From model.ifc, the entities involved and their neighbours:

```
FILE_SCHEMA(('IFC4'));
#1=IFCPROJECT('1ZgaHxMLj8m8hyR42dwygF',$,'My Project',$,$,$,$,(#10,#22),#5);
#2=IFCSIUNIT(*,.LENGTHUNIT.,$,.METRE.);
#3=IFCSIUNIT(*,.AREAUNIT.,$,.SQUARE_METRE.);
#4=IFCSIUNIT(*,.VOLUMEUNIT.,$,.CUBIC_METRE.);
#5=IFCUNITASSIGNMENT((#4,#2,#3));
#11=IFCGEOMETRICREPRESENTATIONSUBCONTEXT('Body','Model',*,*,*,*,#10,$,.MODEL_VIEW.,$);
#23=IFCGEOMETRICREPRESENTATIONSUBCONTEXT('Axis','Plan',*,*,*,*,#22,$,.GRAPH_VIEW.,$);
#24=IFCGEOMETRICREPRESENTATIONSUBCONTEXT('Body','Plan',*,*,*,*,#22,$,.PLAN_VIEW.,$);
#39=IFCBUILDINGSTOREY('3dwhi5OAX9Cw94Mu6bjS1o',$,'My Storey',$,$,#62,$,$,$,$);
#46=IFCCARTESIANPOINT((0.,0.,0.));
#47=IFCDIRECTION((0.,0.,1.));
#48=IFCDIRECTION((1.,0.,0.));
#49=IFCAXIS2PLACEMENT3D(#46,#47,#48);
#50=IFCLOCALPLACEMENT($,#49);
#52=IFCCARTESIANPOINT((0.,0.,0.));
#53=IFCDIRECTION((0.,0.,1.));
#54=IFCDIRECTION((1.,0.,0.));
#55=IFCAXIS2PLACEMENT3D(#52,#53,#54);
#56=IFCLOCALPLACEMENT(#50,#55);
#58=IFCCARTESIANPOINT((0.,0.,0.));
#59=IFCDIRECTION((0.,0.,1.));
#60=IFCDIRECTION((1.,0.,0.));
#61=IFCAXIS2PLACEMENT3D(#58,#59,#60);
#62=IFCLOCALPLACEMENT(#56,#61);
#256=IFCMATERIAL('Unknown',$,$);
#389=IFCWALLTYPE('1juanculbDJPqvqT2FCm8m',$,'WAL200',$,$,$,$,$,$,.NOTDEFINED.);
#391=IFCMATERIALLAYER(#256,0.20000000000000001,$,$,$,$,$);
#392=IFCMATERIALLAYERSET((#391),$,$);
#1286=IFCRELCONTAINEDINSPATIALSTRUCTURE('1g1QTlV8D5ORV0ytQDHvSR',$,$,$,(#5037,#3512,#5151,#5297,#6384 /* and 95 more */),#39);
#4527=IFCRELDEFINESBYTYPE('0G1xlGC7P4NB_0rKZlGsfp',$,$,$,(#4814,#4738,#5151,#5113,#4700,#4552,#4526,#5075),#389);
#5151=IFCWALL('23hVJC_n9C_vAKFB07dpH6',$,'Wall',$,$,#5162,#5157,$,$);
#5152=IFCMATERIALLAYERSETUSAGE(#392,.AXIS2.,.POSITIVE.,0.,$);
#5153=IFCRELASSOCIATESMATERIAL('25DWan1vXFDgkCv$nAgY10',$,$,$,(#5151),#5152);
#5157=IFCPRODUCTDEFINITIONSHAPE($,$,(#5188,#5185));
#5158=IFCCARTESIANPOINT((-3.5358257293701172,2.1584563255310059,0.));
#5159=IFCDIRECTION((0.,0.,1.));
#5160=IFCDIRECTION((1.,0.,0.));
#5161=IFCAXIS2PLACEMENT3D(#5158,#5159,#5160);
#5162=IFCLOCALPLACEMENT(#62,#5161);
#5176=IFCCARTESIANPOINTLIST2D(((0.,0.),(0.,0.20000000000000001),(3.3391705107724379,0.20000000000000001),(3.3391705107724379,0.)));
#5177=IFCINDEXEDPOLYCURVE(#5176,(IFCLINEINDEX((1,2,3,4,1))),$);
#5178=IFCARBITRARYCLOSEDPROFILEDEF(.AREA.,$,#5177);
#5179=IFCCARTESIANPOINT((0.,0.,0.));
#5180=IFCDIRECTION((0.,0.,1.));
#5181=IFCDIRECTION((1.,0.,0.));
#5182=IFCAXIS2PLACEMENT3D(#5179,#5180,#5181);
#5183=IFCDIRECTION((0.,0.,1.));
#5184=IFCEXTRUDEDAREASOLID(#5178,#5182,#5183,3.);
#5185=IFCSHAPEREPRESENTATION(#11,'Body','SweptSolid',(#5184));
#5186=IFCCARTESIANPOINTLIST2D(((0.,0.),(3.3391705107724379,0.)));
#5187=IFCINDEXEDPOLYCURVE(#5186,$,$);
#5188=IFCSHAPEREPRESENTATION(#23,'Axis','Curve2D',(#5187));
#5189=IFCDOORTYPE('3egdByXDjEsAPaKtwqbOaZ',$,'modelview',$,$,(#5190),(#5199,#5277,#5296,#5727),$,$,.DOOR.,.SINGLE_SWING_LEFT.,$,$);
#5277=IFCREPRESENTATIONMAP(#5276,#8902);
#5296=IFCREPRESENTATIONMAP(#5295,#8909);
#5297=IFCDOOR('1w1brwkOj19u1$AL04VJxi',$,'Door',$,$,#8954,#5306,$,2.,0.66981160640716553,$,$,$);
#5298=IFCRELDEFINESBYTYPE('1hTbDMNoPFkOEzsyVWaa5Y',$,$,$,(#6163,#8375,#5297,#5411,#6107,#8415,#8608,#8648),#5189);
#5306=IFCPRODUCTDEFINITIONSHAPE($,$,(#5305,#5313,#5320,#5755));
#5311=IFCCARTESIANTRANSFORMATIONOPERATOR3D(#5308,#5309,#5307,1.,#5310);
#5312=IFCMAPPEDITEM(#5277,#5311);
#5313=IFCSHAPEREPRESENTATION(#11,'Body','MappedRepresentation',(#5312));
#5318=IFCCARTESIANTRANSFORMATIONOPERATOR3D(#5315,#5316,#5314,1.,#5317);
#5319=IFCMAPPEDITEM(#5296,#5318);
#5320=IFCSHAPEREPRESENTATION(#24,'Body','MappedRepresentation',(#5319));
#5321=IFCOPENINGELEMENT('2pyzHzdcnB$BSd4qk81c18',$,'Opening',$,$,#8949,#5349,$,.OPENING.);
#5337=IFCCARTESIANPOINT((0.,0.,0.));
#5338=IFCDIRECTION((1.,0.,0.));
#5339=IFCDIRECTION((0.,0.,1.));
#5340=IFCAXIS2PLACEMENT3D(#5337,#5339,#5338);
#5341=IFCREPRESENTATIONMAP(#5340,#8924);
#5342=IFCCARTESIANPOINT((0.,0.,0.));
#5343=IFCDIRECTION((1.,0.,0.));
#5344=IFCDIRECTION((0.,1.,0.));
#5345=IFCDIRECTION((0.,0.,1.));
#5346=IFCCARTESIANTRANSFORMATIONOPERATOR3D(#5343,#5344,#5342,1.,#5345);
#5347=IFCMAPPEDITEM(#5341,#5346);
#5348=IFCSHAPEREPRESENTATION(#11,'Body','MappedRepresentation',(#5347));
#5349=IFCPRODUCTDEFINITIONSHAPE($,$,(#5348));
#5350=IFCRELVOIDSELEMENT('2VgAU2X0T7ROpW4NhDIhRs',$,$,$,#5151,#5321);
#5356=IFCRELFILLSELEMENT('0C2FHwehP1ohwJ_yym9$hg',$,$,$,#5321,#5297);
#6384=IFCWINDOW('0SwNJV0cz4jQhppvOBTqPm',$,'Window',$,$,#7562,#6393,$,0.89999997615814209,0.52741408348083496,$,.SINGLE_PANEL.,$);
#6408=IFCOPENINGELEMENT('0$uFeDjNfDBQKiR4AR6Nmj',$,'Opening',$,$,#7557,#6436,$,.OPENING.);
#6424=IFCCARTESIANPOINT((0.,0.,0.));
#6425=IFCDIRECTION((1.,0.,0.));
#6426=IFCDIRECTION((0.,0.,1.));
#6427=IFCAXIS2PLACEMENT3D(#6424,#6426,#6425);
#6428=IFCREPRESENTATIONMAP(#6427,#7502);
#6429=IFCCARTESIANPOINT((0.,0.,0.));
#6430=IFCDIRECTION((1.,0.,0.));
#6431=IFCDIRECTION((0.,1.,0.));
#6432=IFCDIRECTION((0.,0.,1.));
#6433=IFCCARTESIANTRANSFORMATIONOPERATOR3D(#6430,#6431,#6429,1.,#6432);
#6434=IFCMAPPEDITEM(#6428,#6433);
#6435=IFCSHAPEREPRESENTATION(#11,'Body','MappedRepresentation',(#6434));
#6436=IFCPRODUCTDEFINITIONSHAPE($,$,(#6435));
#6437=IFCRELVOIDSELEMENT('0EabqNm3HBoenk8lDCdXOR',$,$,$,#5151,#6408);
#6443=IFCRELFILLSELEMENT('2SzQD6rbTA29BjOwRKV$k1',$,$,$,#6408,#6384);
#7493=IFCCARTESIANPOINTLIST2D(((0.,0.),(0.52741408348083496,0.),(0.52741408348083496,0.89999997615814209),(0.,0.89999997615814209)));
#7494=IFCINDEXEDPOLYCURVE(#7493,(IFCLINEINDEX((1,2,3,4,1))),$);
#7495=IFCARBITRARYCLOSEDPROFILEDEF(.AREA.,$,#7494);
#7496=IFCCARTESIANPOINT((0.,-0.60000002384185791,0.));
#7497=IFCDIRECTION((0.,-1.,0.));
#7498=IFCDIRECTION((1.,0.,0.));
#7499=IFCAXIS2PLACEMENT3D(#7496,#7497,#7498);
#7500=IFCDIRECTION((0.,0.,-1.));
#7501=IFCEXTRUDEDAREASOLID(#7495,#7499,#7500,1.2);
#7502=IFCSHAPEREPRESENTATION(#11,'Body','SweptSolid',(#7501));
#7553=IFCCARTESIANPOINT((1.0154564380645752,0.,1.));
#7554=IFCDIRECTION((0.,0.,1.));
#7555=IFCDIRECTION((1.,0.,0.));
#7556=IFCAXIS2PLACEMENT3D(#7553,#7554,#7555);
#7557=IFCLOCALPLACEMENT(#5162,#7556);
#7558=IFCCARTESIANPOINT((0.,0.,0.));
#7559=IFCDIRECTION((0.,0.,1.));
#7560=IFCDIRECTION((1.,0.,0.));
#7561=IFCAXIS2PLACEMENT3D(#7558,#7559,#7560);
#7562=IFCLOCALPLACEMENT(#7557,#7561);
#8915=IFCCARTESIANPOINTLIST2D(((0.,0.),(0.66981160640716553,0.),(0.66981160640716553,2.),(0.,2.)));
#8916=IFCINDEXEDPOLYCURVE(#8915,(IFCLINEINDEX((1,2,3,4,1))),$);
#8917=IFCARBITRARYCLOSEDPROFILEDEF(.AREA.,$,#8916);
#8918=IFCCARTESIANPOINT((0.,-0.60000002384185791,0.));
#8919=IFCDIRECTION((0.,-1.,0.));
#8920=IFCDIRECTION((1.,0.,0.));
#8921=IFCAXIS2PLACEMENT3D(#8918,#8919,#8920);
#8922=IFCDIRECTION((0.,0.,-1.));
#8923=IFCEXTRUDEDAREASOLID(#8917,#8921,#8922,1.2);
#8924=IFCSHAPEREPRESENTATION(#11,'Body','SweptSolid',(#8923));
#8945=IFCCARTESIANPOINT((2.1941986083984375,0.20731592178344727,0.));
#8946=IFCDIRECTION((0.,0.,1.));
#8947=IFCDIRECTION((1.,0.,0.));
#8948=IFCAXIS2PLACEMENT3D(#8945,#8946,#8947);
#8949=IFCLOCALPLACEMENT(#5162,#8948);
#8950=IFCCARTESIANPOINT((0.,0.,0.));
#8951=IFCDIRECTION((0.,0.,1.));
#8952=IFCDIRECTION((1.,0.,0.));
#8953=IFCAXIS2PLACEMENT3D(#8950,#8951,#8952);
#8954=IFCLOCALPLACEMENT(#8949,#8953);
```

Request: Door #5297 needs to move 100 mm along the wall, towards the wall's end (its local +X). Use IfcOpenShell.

```python
import ifcopenshell
import ifcopenshell.api.geometry
import ifcopenshell.util.placement

model = ifcopenshell.open("model.ifc")

door = model.by_guid("1w1brwkOj19u1$AL04VJxi")
opening = door.FillsVoids[0].RelatingOpeningElement
wall = opening.VoidsElements[0].RelatingBuildingElement

wall_matrix = ifcopenshell.util.placement.get_local_placement(wall.ObjectPlacement)
shift = wall_matrix[:3, 0] * 0.1
before = ifcopenshell.util.placement.get_local_placement(door.ObjectPlacement)[:3, 3].copy()

# The door is placed relative to its opening, so it follows when the opening moves.
matrix = ifcopenshell.util.placement.get_local_placement(opening.ObjectPlacement)
matrix[:3, 3] += shift
ifcopenshell.api.geometry.edit_object_placement(
    model, product=opening, matrix=matrix, is_si=False, should_transform_children=True
)

after = ifcopenshell.util.placement.get_local_placement(door.ObjectPlacement)[:3, 3]
print("door moved by", (after - before).round(3) + 0.0)

model.write("model_edited.ifc")
```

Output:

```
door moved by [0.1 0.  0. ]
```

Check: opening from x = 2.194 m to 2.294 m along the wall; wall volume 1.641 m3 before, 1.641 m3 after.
